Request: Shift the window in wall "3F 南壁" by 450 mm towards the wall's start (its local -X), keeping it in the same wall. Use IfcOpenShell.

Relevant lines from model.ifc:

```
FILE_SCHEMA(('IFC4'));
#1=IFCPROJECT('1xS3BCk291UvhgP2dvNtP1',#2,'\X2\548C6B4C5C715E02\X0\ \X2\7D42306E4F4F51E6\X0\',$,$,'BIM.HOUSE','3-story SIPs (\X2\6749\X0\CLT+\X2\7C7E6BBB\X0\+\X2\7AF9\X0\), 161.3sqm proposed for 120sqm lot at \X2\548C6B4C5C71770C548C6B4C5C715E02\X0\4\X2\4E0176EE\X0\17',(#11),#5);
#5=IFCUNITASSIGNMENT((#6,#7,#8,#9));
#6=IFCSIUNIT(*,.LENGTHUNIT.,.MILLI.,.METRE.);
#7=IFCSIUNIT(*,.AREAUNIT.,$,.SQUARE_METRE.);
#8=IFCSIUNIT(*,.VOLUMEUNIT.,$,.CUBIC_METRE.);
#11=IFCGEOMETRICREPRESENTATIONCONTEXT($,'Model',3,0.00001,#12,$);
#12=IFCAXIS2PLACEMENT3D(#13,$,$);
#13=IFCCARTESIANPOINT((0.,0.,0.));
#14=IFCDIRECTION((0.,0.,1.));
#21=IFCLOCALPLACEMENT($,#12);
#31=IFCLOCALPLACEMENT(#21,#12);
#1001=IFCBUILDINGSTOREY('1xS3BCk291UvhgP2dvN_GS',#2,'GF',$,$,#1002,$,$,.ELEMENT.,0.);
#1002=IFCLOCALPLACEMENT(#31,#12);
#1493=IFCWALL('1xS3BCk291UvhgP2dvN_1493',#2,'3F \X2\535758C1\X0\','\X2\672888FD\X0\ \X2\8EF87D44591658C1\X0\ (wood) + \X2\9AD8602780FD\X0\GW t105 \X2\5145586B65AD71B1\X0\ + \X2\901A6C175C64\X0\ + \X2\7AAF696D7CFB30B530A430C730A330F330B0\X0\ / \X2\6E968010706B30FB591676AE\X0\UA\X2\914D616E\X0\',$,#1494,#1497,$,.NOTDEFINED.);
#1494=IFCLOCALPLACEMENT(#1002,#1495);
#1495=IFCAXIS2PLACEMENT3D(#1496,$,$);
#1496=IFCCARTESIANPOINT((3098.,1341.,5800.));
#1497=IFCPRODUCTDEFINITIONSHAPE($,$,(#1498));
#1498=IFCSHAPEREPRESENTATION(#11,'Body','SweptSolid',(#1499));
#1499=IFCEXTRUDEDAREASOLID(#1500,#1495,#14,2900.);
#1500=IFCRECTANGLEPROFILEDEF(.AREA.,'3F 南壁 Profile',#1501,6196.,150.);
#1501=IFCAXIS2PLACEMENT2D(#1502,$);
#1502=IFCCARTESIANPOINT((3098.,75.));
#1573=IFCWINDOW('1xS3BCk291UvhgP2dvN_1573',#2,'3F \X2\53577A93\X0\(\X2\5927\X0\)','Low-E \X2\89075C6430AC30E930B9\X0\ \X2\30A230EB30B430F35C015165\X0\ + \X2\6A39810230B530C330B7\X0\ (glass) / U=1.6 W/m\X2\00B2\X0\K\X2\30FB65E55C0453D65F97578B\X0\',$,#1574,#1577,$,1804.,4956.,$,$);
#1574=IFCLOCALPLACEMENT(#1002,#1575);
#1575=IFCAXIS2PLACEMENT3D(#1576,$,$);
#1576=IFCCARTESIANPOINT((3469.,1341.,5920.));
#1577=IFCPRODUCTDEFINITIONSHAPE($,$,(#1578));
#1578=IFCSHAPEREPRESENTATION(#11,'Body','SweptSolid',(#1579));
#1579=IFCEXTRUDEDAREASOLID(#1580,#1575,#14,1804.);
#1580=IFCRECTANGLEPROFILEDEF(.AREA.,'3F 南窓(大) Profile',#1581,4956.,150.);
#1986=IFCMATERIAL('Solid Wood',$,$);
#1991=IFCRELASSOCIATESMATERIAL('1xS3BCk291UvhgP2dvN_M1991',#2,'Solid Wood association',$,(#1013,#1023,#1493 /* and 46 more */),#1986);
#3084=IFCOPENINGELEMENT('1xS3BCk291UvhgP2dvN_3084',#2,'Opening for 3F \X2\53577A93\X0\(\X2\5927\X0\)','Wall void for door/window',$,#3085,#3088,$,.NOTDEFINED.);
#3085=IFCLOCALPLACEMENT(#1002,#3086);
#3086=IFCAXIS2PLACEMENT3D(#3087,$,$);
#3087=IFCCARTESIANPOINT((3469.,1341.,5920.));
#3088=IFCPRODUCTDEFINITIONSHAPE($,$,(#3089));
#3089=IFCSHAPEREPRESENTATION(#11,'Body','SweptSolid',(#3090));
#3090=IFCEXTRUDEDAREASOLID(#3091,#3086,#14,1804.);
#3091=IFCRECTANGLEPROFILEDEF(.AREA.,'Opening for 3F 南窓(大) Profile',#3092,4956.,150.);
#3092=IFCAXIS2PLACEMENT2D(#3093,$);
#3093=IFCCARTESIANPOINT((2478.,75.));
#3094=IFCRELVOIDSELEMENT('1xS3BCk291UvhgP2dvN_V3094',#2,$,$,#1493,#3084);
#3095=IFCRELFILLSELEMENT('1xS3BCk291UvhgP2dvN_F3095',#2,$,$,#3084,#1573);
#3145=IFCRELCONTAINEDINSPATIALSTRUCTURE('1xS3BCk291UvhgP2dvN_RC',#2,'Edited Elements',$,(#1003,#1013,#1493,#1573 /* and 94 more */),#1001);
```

```python
import ifcopenshell
import ifcopenshell.api.geometry
import ifcopenshell.util.placement
import ifcopenshell.util.unit

model = ifcopenshell.open("model.ifc")
unit_scale = ifcopenshell.util.unit.calculate_unit_scale(model)

window = model.by_id(1573)
opening = window.FillsVoids[0].RelatingOpeningElement
wall = opening.VoidsElements[0].RelatingBuildingElement

wall_matrix = ifcopenshell.util.placement.get_local_placement(wall.ObjectPlacement)
shift = wall_matrix[:3, 0] * -0.45 / unit_scale
before = ifcopenshell.util.placement.get_local_placement(window.ObjectPlacement)[:3, 3].copy()

# The window is not placed relative to its opening, so move both.
for product in (opening, window):
    matrix = ifcopenshell.util.placement.get_local_placement(product.ObjectPlacement)
    matrix[:3, 3] += shift
    ifcopenshell.api.geometry.edit_object_placement(model, product=product, matrix=matrix, is_si=False)

after = ifcopenshell.util.placement.get_local_placement(window.ObjectPlacement)[:3, 3]
print("window moved by", (after - before).round(3) + 0.0)

model.write("model_v2.ifc")
```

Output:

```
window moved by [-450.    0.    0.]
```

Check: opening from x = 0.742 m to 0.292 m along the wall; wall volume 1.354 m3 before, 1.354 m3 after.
